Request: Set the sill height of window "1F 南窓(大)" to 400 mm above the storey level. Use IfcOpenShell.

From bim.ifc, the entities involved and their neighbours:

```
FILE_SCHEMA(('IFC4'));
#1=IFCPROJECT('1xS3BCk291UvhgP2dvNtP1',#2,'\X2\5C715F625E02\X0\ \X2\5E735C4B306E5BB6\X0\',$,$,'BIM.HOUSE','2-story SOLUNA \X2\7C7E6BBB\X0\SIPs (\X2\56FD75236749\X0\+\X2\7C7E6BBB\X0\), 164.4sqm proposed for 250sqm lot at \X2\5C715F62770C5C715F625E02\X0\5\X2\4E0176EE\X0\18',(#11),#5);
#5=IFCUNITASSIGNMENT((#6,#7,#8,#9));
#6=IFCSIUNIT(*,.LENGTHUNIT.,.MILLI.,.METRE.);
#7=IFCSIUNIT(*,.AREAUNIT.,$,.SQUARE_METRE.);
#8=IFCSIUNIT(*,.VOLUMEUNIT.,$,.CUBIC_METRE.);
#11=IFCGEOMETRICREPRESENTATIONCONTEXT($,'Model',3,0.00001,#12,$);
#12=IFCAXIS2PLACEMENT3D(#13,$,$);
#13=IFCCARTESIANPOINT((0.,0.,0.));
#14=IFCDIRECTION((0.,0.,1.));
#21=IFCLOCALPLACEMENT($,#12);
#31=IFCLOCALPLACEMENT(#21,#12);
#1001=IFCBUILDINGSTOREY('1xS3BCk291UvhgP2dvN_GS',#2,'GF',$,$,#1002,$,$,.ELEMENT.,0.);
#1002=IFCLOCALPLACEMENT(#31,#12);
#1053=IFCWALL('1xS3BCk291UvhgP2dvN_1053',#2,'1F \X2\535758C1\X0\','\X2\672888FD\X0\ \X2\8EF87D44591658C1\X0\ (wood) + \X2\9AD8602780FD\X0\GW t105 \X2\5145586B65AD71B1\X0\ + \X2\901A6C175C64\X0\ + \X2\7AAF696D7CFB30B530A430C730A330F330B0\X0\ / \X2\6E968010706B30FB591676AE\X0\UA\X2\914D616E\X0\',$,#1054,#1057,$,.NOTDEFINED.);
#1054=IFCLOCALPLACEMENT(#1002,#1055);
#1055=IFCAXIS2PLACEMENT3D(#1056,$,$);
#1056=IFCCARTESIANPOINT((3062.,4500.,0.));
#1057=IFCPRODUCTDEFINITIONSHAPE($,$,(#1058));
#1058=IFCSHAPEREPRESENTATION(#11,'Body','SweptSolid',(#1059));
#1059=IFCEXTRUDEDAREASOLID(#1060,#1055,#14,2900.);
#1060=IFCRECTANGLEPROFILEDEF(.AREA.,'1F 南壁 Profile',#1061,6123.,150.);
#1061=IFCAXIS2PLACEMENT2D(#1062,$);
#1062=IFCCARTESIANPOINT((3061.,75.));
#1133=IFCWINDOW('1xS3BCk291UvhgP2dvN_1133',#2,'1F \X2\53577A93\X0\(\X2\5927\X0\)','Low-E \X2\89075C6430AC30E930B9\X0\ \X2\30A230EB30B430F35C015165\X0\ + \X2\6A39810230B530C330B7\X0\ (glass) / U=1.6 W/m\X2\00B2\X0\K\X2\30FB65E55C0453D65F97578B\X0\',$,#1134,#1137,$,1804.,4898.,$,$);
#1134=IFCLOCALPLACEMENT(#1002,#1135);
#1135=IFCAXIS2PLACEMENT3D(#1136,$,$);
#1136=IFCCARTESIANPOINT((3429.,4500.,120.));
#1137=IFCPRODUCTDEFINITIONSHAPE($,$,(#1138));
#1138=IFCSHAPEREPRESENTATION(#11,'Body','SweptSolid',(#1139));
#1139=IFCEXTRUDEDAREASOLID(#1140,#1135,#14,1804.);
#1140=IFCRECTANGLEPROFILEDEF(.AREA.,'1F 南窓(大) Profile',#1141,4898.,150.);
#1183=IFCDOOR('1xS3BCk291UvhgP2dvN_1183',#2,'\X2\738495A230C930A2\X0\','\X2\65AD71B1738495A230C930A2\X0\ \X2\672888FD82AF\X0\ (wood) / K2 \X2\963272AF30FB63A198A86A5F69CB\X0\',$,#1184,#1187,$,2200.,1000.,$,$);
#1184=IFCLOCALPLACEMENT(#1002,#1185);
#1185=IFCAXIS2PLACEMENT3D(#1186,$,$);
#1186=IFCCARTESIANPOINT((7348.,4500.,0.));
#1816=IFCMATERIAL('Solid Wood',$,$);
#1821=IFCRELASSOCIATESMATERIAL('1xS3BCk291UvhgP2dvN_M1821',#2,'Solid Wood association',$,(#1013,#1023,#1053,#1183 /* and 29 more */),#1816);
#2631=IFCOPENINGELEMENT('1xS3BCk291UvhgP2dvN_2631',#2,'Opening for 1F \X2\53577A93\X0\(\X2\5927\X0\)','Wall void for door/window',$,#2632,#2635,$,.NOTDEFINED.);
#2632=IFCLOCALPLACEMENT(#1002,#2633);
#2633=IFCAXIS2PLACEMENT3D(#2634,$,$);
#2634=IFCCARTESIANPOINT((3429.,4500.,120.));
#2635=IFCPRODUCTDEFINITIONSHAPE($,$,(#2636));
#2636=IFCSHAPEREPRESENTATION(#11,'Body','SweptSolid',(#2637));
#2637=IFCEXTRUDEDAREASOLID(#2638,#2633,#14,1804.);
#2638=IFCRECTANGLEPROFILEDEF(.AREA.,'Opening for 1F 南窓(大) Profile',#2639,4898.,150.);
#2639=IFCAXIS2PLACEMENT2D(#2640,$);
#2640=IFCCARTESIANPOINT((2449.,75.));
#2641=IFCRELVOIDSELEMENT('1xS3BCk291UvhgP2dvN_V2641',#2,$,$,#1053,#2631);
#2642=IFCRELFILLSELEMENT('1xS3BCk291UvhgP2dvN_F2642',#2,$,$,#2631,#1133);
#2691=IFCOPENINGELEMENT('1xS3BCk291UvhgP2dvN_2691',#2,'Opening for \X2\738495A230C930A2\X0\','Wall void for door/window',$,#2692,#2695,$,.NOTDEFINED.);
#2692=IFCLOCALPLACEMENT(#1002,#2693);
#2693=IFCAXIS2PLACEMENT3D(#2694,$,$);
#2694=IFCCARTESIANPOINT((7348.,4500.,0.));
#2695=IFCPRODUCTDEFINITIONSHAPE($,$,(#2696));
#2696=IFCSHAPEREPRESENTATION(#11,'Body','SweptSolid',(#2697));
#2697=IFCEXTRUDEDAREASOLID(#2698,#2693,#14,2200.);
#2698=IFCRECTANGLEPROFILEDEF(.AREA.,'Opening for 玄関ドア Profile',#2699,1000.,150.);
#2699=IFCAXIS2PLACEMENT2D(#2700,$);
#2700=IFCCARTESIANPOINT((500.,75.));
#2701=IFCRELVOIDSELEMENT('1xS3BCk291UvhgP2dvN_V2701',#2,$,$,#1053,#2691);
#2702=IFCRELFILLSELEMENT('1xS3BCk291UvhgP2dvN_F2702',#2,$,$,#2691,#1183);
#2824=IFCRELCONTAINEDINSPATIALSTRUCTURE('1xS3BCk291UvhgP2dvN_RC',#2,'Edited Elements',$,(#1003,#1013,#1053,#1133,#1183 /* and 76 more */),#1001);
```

```python
import numpy as np
import ifcopenshell
import ifcopenshell.api.geometry
import ifcopenshell.geom
import ifcopenshell.util.element
import ifcopenshell.util.placement
import ifcopenshell.util.shape
import ifcopenshell.util.unit

model = ifcopenshell.open("bim.ifc")
unit_scale = ifcopenshell.util.unit.calculate_unit_scale(model)

window = model.by_guid("1xS3BCk291UvhgP2dvN_1133")
opening = window.FillsVoids[0].RelatingOpeningElement
storey = ifcopenshell.util.element.get_container(window, ifc_class="IfcBuildingStorey")
level = ifcopenshell.util.placement.get_local_placement(storey.ObjectPlacement)[2, 3]

# The opening's origin need not be at the sill, so measure its lowest point.
shape = ifcopenshell.geom.create_shape(ifcopenshell.geom.settings(), opening)
bottom = ifcopenshell.util.shape.get_shape_bottom_elevation(shape, shape.geometry) / unit_scale
dz = level + 0.4 / unit_scale - bottom

shift = np.array([0.0, 0.0, dz])
# The window is not placed relative to its opening, so move both.
for product in (opening, window):
    matrix = ifcopenshell.util.placement.get_local_placement(product.ObjectPlacement)
    matrix[:3, 3] += shift
    ifcopenshell.api.geometry.edit_object_placement(model, product=product, matrix=matrix, is_si=False)

print(f"moved by {dz * unit_scale:+.3f} m")

model.write("bim-out.ifc")
```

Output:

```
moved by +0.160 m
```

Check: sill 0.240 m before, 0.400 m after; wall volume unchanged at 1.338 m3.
